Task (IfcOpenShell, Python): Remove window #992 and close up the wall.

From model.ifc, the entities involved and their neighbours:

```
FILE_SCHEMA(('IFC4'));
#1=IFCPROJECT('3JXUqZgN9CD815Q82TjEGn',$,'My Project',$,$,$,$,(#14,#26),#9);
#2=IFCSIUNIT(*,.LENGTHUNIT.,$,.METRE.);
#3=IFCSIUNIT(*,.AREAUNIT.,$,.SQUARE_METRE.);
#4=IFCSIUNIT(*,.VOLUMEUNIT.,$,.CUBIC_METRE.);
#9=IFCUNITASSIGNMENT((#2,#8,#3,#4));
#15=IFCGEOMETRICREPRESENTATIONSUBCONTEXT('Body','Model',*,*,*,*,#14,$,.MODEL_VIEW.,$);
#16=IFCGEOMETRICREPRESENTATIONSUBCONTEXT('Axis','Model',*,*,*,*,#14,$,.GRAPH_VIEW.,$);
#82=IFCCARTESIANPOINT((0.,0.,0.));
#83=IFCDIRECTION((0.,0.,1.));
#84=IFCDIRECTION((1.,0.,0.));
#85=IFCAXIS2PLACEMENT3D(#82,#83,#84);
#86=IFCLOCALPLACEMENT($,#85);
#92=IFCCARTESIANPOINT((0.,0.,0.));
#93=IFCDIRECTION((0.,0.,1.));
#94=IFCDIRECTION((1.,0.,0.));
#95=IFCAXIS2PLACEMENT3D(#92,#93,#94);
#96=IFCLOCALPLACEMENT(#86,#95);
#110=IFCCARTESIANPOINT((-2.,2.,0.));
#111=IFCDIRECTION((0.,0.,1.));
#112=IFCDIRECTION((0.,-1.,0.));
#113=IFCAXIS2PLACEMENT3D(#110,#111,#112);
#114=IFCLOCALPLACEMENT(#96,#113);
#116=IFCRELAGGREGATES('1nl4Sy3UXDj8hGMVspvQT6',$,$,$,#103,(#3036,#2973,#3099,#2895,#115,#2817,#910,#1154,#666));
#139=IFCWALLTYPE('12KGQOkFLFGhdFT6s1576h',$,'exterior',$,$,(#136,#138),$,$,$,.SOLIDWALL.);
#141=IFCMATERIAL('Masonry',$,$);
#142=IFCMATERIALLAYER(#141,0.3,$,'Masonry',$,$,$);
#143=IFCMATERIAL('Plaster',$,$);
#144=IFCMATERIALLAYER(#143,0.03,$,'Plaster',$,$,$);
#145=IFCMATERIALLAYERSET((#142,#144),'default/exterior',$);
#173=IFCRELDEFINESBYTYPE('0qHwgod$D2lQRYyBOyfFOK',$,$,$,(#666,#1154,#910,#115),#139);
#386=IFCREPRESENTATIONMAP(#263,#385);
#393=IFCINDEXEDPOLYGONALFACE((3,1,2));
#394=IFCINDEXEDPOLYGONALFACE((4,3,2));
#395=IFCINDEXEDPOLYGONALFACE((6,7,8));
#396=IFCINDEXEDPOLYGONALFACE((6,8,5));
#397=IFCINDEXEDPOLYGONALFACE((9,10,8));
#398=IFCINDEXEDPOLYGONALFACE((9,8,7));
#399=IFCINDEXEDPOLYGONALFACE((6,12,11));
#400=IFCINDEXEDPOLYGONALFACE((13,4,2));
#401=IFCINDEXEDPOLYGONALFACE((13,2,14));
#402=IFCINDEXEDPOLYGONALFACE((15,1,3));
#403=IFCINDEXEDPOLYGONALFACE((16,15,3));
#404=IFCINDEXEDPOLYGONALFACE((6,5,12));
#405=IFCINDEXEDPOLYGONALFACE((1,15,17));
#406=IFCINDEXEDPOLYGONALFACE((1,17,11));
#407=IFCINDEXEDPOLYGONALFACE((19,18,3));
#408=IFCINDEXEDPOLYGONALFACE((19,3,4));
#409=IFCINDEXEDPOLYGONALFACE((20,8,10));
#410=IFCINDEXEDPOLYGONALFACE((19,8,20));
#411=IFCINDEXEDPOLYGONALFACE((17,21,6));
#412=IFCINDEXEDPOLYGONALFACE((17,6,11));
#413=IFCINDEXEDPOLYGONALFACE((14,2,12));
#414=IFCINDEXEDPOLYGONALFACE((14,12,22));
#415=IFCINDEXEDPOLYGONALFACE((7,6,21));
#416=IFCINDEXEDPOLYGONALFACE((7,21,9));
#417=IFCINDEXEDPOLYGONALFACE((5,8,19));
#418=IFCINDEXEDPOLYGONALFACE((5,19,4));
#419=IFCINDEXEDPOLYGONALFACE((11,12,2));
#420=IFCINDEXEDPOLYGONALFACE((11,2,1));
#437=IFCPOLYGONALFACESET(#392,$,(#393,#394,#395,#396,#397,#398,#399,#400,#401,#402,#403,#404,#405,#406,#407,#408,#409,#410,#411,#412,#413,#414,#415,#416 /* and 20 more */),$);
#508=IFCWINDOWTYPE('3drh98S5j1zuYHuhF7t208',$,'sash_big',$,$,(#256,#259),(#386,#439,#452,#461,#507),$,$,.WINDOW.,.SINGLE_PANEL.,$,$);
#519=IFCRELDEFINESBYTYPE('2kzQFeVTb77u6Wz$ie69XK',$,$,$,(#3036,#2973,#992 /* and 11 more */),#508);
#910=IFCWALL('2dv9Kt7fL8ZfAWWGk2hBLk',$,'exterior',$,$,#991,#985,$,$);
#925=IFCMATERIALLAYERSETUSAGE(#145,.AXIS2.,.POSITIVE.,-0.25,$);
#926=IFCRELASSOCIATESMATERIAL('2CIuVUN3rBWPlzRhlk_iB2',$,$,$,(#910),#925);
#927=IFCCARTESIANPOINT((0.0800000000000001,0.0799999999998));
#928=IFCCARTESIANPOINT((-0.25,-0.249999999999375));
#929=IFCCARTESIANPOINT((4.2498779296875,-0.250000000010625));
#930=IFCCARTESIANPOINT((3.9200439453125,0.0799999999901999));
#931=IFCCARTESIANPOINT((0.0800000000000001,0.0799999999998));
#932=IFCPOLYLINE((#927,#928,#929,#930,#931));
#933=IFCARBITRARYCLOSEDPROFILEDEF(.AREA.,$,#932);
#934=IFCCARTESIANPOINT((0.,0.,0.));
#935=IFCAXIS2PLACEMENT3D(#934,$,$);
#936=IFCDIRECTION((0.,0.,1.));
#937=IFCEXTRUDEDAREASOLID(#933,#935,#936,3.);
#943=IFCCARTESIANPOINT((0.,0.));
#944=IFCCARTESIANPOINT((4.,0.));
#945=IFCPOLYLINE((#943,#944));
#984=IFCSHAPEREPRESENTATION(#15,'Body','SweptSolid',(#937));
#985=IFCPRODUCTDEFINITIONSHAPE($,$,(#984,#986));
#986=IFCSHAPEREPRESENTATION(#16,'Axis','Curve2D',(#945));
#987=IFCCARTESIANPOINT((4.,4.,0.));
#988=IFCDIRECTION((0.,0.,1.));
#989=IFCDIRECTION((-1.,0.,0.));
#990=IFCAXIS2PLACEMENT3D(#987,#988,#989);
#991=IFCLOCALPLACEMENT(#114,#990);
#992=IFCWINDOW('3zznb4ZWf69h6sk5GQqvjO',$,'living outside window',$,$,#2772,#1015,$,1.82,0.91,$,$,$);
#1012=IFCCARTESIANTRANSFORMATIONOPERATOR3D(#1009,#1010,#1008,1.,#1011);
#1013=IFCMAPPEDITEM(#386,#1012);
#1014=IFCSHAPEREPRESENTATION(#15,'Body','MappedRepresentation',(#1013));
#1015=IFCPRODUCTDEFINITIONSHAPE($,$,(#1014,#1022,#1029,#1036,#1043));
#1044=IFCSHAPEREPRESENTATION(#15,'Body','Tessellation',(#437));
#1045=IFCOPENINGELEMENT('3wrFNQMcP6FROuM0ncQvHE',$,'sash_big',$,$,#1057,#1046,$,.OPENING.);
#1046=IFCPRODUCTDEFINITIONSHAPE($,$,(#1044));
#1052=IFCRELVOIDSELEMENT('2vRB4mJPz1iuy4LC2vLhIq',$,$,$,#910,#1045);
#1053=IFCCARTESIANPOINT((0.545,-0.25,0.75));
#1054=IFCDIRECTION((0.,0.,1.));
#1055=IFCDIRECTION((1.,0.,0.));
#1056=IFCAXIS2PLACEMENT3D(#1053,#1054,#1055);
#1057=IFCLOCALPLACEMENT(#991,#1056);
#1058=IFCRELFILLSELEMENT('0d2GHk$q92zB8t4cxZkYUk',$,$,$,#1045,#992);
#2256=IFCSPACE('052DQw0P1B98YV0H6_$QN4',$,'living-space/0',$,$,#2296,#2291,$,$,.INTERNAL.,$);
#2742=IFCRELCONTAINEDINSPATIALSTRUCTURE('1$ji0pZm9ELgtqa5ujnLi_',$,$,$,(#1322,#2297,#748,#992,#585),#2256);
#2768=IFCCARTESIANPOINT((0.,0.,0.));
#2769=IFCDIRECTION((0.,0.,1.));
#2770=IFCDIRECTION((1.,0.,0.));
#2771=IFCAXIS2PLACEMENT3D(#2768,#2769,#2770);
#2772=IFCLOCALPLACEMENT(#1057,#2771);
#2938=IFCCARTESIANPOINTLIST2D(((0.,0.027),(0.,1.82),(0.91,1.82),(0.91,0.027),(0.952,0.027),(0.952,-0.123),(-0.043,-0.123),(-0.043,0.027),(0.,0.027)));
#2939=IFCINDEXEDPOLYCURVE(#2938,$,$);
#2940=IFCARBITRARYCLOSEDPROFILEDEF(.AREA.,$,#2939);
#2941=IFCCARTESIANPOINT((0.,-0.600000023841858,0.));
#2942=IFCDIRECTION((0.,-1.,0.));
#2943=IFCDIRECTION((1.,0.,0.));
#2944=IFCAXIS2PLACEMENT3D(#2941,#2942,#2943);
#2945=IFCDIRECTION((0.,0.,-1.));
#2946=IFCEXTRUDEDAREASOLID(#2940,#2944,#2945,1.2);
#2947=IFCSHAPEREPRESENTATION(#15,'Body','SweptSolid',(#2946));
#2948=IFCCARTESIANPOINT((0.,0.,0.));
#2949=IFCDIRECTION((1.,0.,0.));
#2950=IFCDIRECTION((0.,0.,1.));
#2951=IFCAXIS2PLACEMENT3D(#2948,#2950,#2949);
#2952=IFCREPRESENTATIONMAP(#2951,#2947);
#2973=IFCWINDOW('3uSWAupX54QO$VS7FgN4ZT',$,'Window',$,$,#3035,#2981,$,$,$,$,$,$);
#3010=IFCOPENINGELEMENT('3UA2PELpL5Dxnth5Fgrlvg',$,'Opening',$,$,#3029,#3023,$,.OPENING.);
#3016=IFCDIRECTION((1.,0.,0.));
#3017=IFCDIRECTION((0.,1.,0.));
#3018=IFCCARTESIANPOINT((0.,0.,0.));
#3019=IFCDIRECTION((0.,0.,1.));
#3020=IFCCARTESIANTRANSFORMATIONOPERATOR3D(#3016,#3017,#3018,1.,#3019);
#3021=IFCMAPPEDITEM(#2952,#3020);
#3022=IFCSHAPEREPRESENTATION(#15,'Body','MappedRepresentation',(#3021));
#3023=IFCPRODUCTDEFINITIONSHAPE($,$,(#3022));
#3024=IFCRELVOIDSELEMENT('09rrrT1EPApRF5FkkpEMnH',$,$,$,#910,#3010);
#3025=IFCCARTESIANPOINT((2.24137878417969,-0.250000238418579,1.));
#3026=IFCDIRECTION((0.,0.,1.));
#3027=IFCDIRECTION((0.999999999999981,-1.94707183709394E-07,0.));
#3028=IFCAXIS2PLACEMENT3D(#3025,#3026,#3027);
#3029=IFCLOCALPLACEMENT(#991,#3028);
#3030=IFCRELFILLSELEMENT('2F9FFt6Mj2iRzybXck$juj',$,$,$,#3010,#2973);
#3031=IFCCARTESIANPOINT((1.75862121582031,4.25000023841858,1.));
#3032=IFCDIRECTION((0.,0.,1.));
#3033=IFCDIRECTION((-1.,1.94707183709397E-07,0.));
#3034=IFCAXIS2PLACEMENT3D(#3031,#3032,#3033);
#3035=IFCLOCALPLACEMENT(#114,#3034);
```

```python
import ifcopenshell
import ifcopenshell.api.feature
import ifcopenshell.api.root
import ifcopenshell.geom
import ifcopenshell.util.shape

model = ifcopenshell.open("model.ifc")
settings = ifcopenshell.geom.settings()


def volume(element):
    """Net volume in cubic metres, openings subtracted."""
    shape = ifcopenshell.geom.create_shape(settings, element)
    return ifcopenshell.util.shape.get_volume(shape.geometry)


window = model.by_guid("3zznb4ZWf69h6sk5GQqvjO")
opening = window.FillsVoids[0].RelatingOpeningElement
wall = opening.VoidsElements[0].RelatingBuildingElement
before = volume(wall)

ifcopenshell.api.root.remove_product(model, product=window)
ifcopenshell.api.feature.remove_feature(model, feature=opening)

after = volume(wall)

print(f"wall volume {before:.3f} -> {after:.3f} m3")

model.write("model-out.ifc")
```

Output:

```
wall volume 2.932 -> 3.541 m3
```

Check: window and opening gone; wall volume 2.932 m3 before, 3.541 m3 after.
